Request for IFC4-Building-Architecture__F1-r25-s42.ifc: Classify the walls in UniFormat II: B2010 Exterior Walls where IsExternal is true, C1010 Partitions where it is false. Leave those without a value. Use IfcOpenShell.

First a look at what the model holds.

```python
import ifcopenshell
import ifcopenshell.util.element

model = ifcopenshell.open("IFC4-Building-Architecture__F1-r25-s42.ifc")
print(model.schema)
print("classifications:", [c.Name for c in model.by_type("IfcClassification")])
values = [ifcopenshell.util.element.get_pset(e, "Pset_WallCommon", "IsExternal") for e in model.by_type("IfcWall")]
for value in (True, False, None):
    print("IsExternal", value, values.count(value))
```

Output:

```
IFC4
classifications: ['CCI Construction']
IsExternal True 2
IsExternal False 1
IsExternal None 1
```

```python
import ifcopenshell
import ifcopenshell.api.classification
import ifcopenshell.util.element

model = ifcopenshell.open("IFC4-Building-Architecture__F1-r25-s42.ifc")

system = ifcopenshell.api.classification.add_classification(model, classification="UniFormat II")

walls = model.by_type("IfcWall")
external = {e: ifcopenshell.util.element.get_pset(e, "Pset_WallCommon", "IsExternal") for e in walls}
for flag, code, name in ((True, "B2010", "Exterior Walls"), (False, "C1010", "Partitions")):
    products = [e for e in walls if external[e] is flag]
    ifcopenshell.api.classification.add_reference(
        model, products=products, classification=system, identification=code, name=name
    )
    print(code, len(products))

model.write("IFC4-Building-Architecture__F1-r25-s42-out.ifc")
```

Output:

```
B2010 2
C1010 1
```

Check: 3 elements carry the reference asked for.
